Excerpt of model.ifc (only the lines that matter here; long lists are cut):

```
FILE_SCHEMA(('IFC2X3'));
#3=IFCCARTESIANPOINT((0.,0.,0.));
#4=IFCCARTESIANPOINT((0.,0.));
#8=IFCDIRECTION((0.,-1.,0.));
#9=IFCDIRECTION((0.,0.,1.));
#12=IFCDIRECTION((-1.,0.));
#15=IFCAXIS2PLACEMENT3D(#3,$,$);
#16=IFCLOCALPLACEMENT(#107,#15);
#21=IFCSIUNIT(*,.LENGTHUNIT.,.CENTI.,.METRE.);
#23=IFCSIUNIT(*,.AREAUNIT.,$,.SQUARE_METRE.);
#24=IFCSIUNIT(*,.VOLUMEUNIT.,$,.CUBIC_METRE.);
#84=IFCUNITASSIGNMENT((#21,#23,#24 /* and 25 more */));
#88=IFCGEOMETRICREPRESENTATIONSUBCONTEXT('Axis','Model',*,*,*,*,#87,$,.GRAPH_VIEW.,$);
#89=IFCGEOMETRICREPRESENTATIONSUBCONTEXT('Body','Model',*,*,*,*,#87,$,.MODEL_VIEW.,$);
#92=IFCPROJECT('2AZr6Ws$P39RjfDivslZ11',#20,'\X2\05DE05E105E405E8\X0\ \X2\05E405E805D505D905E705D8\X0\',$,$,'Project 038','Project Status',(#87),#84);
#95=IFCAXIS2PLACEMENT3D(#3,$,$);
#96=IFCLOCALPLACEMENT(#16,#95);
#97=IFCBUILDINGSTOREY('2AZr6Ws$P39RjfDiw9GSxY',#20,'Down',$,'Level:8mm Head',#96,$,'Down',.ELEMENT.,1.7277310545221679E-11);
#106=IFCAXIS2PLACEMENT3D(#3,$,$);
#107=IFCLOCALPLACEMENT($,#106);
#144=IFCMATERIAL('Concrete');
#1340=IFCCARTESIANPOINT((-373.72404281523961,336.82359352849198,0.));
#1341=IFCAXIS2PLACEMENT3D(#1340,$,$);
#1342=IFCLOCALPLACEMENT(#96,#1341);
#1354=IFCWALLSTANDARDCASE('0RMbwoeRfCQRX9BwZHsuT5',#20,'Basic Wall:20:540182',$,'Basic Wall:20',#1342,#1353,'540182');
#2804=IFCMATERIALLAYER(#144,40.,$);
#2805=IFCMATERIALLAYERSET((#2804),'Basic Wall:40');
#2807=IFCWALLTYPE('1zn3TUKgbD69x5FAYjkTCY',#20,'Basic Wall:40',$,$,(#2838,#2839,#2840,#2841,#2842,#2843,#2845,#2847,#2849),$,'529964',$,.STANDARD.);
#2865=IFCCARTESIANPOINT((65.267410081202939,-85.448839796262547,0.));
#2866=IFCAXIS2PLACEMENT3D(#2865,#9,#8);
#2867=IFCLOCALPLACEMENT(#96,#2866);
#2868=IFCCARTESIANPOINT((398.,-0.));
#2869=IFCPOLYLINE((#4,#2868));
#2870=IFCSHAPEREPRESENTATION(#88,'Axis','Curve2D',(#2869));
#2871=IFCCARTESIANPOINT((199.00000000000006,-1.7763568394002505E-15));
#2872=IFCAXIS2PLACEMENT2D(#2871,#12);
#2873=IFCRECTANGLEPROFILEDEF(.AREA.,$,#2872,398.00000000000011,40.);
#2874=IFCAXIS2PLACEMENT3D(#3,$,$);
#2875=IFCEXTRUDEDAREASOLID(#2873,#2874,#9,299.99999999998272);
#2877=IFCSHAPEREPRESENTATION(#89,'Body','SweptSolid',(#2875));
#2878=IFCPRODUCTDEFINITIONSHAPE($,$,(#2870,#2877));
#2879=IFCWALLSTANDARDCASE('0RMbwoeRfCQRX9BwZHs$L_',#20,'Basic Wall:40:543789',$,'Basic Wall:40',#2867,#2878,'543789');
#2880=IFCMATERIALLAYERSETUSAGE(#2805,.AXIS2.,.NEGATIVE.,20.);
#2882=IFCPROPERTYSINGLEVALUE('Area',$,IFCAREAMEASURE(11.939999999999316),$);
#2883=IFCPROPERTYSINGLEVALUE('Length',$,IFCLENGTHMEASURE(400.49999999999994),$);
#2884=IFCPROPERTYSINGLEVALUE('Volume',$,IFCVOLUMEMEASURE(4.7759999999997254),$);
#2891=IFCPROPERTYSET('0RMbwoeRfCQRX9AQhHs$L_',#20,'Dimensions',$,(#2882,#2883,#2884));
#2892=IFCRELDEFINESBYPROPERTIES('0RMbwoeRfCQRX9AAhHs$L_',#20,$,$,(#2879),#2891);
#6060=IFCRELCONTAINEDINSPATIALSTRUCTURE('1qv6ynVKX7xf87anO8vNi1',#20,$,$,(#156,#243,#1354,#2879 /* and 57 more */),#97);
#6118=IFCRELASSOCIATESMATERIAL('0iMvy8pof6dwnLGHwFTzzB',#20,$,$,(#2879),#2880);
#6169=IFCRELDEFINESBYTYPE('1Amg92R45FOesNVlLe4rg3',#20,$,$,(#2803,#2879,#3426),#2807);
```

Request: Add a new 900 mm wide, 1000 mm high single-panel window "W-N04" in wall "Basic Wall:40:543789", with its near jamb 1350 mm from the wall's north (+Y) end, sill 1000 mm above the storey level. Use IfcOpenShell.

```python
import numpy as np
import ifcopenshell
import ifcopenshell.api.feature
import ifcopenshell.api.geometry
import ifcopenshell.api.pset
import ifcopenshell.api.root
import ifcopenshell.api.spatial
import ifcopenshell.api.type
import ifcopenshell.geom
import ifcopenshell.util.element
import ifcopenshell.util.placement
import ifcopenshell.util.representation
import ifcopenshell.util.shape
import ifcopenshell.util.unit

model = ifcopenshell.open("model.ifc")
unit_scale = ifcopenshell.util.unit.calculate_unit_scale(model)
area_scale = ifcopenshell.util.unit.calculate_unit_scale(model, "AREAUNIT")
volume_scale = ifcopenshell.util.unit.calculate_unit_scale(model, "VOLUMEUNIT")
settings = ifcopenshell.geom.settings()


def volume(element):
    """Net volume in cubic metres, openings subtracted."""
    shape = ifcopenshell.geom.create_shape(settings, element)
    return ifcopenshell.util.shape.get_volume(shape.geometry)


wall = model.by_guid("0RMbwoeRfCQRX9BwZHs$L_")
storey = ifcopenshell.util.element.get_container(wall, ifc_class="IfcBuildingStorey")
context = ifcopenshell.util.representation.get_context(model, "Model", "Body", "MODEL_VIEW")
before = volume(wall)

width, height, from_end, sill = 0.9, 1, 1.35, 1  # metres

# The wall runs along its own X axis, and the end named is its -X end.
wall_shape = ifcopenshell.geom.create_shape(settings, wall)
x, y, z = ifcopenshell.util.shape.get_vertices(wall_shape.geometry).T
start = x.min() + from_end
face, thickness = float(y.min()), float(y.max() - y.min())
wall_matrix = ifcopenshell.util.placement.get_local_placement(wall.ObjectPlacement)
level = ifcopenshell.util.placement.get_local_placement(storey.ObjectPlacement)[2, 3]


def in_wall(x, y):
    """Placement at x, y metres in the wall's axes, at sill height."""
    matrix = wall_matrix.copy()
    matrix[:, 3] = wall_matrix @ np.array([x / unit_scale, y / unit_scale, 0.0, 1.0])
    matrix[2, 3] = level + sill / unit_scale
    return matrix


# Opening: a box that overshoots both wall faces by 50 mm.
opening = ifcopenshell.api.root.create_entity(model, ifc_class="IfcOpeningElement")
box = ifcopenshell.api.geometry.add_wall_representation(
    model, context=context, length=width, height=height, thickness=thickness + 0.1
)
ifcopenshell.api.geometry.assign_representation(model, product=opening, representation=box)
ifcopenshell.api.geometry.edit_object_placement(model, product=opening, matrix=in_wall(start, face - 0.05), is_si=False)
ifcopenshell.api.feature.add_feature(model, feature=opening, element=wall)

window = ifcopenshell.api.root.create_entity(model, ifc_class="IfcWindow", name="W-N04")
window.OverallWidth, window.OverallHeight = width / unit_scale, height / unit_scale
body = ifcopenshell.api.geometry.add_window_representation(
    model,
    context=context,
    overall_width=window.OverallWidth,
    overall_height=window.OverallHeight,
    partition_type="SINGLE_PANEL",
)
ifcopenshell.api.geometry.assign_representation(model, product=window, representation=body)
ifcopenshell.api.spatial.assign_container(model, products=[window], relating_structure=storey)
fills = ifcopenshell.api.feature.add_filling(model, opening=opening, element=window)
fills.OwnerHistory = window.OwnerHistory  # required in IFC2X3

# IFC2X3 keeps the operation on the window style.
style = ifcopenshell.api.root.create_entity(model, ifc_class="IfcWindowStyle", name="W-N04")
style.OperationType, style.ConstructionType = "SINGLE_PANEL", "NOTDEFINED"
style.ParameterTakesPrecedence = style.Sizeable = False
ifcopenshell.api.type.assign_type(model, related_objects=[window], relating_type=style)

# Centre the window in the wall's thickness.
ifcopenshell.api.geometry.edit_object_placement(model, product=window, matrix=in_wall(start, face), is_si=False)
window_shape = ifcopenshell.geom.create_shape(settings, window)
depth = ifcopenshell.util.shape.get_vertices(window_shape.geometry)[:, 1]
offset = face + thickness / 2 - (depth.min() + depth.max()) / 2
ifcopenshell.api.geometry.edit_object_placement(model, product=window, matrix=in_wall(start, offset), is_si=False)

after = volume(wall)

# Update the wall's stored quantities.
pset = model.by_id(ifcopenshell.util.element.get_pset(wall, "Dimensions", should_inherit=False)["id"])
ifcopenshell.api.pset.edit_pset(model, pset=pset, properties={
    "Area": model.create_entity("IfcAreaMeasure", after / thickness / area_scale),
    "Volume": model.create_entity("IfcVolumeMeasure", after / volume_scale),
})

print(f"wall volume {before:.3f} -> {after:.3f} m3")

model.write("model_updated.ifc")
```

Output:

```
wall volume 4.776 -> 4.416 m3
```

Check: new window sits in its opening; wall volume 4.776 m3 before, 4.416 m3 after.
